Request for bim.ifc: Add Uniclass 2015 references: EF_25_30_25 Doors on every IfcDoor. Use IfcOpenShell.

First a look at what the model holds.

```python
import ifcopenshell

model = ifcopenshell.open("bim.ifc")
print(model.schema)
print("classifications:", [c.Name for c in model.by_type("IfcClassification")])
for ifc_class in ("IfcDoor", "IfcRoof", "IfcStair", "IfcWall", "IfcWindow"):
    print(ifc_class, len(model.by_type(ifc_class)))
```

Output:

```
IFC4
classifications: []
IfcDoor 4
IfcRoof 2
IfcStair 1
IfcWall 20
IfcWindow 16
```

```python
import ifcopenshell
import ifcopenshell.api.classification

model = ifcopenshell.open("bim.ifc")

system = ifcopenshell.api.classification.add_classification(model, classification="Uniclass 2015")

codes = {
    "IfcDoor": ("EF_25_30_25", "Doors"),
}
for ifc_class, (code, name) in codes.items():
    products = model.by_type(ifc_class)
    ifcopenshell.api.classification.add_reference(
        model, products=products, classification=system, identification=code, name=name
    )
    print(code, len(products))

model.write("bim_edited.ifc")
```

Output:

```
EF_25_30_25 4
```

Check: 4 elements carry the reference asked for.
